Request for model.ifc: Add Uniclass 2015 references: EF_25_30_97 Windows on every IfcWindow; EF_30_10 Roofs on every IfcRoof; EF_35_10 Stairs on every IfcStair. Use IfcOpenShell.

First a look at what the model holds.

```python
import ifcopenshell

model = ifcopenshell.open("model.ifc")
print(model.schema)
print("classifications:", [c.Name for c in model.by_type("IfcClassification")])
for ifc_class in ("IfcDoor", "IfcRoof", "IfcStair", "IfcWall", "IfcWindow"):
    print(ifc_class, len(model.by_type(ifc_class)))
```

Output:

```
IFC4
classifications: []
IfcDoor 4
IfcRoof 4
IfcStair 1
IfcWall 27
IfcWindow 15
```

```python
import ifcopenshell
import ifcopenshell.api.classification

model = ifcopenshell.open("model.ifc")

system = ifcopenshell.api.classification.add_classification(model, classification="Uniclass 2015")

codes = {
    "IfcWindow": ("EF_25_30_97", "Windows"),
    "IfcRoof": ("EF_30_10", "Roofs"),
    "IfcStair": ("EF_35_10", "Stairs"),
}
for ifc_class, (code, name) in codes.items():
    products = model.by_type(ifc_class)
    ifcopenshell.api.classification.add_reference(
        model, products=products, classification=system, identification=code, name=name
    )
    print(code, len(products))

model.write("model_edited.ifc")
```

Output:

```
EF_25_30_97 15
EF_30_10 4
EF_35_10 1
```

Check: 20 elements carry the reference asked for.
